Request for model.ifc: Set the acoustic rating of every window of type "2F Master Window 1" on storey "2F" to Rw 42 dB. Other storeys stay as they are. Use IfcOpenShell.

First a look at what the model holds.

```python
import ifcopenshell
import ifcopenshell.util.element

model = ifcopenshell.open("model.ifc")
print(model.schema)
storey = next(s for s in model.by_type("IfcBuildingStorey") if s.Name == "2F")
windows = [e for e in ifcopenshell.util.element.get_decomposition(storey) if e.is_a("IfcWindow")]
seen = {}
for e in windows:
    element_type = ifcopenshell.util.element.get_type(e)
    key = (element_type.Name if element_type != e and element_type else None, ifcopenshell.util.element.get_pset(e, "Pset_WindowCommon", "AcousticRating"))
    seen[key] = seen.get(key, 0) + 1
for (name, value), count in sorted(seen.items(), key=str):
    print(count, "x", name, "|", value)
```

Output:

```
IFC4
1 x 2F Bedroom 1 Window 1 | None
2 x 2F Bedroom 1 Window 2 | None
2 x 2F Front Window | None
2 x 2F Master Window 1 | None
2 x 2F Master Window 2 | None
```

```python
import ifcopenshell
import ifcopenshell.api.pset
import ifcopenshell.util.element

model = ifcopenshell.open("model.ifc")

storey = next(s for s in model.by_type("IfcBuildingStorey") if s.Name == "2F")
windows = [e for e in ifcopenshell.util.element.get_decomposition(storey) if e.is_a("IfcWindow")]

count = 0
for e in windows:
    element_type = ifcopenshell.util.element.get_type(e)
    if element_type in (None, e) or element_type.Name != "2F Master Window 1":
        continue
    # add_pset returns the element's existing set when there is one.
    pset = ifcopenshell.api.pset.add_pset(model, product=e, name="Pset_WindowCommon")
    ifcopenshell.api.pset.edit_pset(model, pset=pset, properties={"AcousticRating": "Rw 42 dB"})
    count += 1

print(count, "windows updated")

model.write("model_v2.ifc")
```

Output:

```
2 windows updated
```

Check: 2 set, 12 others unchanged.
